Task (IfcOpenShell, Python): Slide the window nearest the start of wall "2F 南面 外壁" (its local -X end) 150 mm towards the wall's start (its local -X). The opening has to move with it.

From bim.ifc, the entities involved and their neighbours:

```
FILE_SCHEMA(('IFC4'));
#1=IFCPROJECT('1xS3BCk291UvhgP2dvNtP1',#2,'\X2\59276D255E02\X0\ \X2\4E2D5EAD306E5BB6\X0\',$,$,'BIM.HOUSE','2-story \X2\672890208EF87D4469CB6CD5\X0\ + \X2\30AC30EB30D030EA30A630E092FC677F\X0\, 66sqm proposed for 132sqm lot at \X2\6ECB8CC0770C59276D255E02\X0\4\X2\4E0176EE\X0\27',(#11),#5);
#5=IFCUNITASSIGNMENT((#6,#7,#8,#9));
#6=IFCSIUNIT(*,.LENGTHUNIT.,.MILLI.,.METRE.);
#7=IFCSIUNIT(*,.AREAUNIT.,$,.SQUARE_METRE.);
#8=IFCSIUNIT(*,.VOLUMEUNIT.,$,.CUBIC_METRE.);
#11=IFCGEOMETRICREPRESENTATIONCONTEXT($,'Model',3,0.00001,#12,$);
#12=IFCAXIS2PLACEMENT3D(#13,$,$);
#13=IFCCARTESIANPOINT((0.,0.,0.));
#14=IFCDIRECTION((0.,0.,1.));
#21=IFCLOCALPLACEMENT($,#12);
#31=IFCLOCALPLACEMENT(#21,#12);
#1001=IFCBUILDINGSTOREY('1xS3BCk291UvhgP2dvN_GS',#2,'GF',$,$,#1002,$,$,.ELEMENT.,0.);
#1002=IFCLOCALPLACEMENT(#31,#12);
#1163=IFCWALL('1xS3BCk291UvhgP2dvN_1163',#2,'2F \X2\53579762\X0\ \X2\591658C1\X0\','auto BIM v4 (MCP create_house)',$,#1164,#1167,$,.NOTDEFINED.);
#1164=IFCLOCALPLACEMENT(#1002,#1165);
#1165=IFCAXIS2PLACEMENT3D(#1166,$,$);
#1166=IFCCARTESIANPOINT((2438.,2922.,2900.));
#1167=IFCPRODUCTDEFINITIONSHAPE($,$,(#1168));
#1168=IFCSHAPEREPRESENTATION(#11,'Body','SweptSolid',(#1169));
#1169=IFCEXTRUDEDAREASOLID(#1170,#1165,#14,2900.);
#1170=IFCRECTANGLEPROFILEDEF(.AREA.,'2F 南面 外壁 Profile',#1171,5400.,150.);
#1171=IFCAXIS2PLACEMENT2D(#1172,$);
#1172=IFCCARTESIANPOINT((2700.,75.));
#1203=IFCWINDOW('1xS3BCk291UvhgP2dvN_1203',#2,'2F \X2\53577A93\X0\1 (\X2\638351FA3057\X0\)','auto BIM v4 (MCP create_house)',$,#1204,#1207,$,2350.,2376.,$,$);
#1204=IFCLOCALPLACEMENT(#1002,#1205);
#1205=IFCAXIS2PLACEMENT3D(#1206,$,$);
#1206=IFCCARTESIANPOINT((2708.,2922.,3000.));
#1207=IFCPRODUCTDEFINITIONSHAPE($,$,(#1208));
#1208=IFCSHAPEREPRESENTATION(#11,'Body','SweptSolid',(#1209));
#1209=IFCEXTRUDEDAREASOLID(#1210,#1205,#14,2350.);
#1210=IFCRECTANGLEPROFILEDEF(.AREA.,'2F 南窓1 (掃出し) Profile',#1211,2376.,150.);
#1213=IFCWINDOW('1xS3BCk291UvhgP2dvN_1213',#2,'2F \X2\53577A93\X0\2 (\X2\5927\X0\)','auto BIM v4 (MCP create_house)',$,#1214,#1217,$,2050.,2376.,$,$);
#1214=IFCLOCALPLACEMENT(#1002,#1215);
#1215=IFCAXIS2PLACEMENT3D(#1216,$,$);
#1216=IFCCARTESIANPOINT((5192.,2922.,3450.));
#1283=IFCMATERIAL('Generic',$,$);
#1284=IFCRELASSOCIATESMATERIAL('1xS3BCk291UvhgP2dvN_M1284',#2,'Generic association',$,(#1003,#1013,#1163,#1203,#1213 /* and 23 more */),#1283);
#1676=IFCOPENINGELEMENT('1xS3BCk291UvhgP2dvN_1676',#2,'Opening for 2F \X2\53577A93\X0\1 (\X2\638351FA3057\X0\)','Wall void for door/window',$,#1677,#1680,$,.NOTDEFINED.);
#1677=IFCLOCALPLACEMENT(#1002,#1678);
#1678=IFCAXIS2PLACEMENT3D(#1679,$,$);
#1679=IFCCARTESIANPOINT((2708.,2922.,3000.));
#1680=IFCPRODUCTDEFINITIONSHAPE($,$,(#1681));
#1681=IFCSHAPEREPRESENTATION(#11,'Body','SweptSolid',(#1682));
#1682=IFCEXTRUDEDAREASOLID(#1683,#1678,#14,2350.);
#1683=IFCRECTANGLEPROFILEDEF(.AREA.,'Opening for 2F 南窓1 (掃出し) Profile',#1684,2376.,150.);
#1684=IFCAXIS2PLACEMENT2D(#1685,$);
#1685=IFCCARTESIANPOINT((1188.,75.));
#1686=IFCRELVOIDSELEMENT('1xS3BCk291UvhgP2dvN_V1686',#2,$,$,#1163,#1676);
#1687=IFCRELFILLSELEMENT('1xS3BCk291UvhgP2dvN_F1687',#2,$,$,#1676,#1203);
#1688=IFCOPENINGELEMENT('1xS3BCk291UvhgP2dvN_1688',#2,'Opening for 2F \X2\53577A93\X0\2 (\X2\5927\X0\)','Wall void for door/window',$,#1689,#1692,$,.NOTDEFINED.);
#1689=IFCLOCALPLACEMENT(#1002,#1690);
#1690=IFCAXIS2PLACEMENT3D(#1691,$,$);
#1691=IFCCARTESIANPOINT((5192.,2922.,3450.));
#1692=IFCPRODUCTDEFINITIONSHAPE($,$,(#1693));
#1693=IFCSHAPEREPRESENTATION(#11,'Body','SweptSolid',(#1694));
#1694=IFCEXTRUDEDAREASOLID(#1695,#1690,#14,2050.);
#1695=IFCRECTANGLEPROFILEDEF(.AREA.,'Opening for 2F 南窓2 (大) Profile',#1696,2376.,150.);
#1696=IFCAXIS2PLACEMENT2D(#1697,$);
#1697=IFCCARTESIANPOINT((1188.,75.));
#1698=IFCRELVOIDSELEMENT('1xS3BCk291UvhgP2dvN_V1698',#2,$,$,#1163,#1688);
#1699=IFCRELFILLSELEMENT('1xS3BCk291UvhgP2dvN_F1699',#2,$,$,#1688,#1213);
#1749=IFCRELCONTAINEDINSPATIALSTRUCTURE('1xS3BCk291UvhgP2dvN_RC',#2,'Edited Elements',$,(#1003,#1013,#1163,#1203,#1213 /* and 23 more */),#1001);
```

```python
import ifcopenshell
import ifcopenshell.api.geometry
import ifcopenshell.util.placement
import ifcopenshell.util.unit

model = ifcopenshell.open("bim.ifc")
unit_scale = ifcopenshell.util.unit.calculate_unit_scale(model)

window = model.by_guid("1xS3BCk291UvhgP2dvN_1203")
opening = window.FillsVoids[0].RelatingOpeningElement
wall = opening.VoidsElements[0].RelatingBuildingElement

wall_matrix = ifcopenshell.util.placement.get_local_placement(wall.ObjectPlacement)
shift = wall_matrix[:3, 0] * -0.15 / unit_scale
before = ifcopenshell.util.placement.get_local_placement(window.ObjectPlacement)[:3, 3].copy()

# The window is not placed relative to its opening, so move both.
for product in (opening, window):
    matrix = ifcopenshell.util.placement.get_local_placement(product.ObjectPlacement)
    matrix[:3, 3] += shift
    ifcopenshell.api.geometry.edit_object_placement(model, product=product, matrix=matrix, is_si=False)

after = ifcopenshell.util.placement.get_local_placement(window.ObjectPlacement)[:3, 3]
print("window moved by", (after - before).round(3) + 0.0)

model.write("bim_edited.ifc")
```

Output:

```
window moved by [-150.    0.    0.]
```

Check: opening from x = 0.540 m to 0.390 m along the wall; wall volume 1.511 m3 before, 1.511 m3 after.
